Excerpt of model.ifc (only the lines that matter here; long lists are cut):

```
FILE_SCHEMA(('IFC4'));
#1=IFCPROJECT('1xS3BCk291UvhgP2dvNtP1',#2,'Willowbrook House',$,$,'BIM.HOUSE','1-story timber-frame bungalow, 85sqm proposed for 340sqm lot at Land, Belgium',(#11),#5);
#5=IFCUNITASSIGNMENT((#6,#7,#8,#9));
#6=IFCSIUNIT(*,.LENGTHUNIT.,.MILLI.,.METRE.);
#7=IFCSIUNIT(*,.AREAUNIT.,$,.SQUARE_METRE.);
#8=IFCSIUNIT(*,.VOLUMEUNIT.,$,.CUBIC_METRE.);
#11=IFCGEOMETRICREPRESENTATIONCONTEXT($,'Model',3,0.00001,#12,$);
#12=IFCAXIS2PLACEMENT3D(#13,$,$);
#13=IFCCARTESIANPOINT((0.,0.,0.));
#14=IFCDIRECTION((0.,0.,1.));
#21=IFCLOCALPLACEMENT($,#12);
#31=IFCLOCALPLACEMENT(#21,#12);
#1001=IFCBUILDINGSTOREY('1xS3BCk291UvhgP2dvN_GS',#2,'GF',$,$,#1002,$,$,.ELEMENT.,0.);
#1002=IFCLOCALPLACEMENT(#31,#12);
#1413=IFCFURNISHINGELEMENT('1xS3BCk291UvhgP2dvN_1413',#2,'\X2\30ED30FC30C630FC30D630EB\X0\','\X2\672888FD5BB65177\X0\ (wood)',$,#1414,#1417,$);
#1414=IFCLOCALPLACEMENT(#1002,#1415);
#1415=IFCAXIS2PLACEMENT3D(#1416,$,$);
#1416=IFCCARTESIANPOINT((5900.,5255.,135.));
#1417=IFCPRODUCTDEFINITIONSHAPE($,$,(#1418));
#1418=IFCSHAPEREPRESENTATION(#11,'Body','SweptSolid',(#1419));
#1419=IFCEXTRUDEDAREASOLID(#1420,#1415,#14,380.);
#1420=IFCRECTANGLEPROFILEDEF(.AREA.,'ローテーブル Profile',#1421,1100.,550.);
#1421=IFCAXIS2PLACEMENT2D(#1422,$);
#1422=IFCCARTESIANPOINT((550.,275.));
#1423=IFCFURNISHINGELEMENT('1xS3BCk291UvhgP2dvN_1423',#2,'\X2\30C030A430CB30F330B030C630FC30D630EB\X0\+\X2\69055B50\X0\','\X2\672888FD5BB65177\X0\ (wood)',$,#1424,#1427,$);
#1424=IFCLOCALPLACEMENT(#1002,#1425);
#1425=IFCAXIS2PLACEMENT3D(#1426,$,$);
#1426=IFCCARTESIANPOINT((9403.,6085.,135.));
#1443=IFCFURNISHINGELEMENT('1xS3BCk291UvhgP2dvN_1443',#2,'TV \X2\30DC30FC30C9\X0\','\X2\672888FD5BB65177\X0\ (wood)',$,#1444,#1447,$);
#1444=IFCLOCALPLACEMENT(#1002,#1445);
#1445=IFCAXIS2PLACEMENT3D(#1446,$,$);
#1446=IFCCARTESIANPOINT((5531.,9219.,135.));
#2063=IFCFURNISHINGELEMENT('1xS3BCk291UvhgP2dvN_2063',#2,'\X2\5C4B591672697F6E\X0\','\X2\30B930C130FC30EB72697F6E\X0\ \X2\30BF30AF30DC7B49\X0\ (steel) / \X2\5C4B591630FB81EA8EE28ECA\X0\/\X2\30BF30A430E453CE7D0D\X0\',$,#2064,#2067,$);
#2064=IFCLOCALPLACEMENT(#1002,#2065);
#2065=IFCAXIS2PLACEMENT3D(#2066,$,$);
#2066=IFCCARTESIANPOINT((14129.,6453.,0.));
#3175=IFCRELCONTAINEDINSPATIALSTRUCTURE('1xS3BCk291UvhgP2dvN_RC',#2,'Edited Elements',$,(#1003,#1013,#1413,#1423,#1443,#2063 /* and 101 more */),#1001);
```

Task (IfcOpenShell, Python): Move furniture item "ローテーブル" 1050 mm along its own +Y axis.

```python
import ifcopenshell
import ifcopenshell.api.geometry
import ifcopenshell.util.placement

model = ifcopenshell.open("model.ifc")

item = model.by_guid("1xS3BCk291UvhgP2dvN_1413")
matrix = ifcopenshell.util.placement.get_local_placement(item.ObjectPlacement)
matrix[:3, 3] += matrix[:3, 1] * 1050.0
ifcopenshell.api.geometry.edit_object_placement(model, product=item, matrix=matrix, is_si=False)

print(ifcopenshell.util.placement.get_local_placement(item.ObjectPlacement).round(3) + 0.0)

model.write("model_rev.ifc")
```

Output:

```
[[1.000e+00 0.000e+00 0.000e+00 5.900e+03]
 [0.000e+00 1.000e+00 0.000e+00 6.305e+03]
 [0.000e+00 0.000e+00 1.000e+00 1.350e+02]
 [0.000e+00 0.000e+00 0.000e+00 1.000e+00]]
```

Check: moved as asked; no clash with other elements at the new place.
